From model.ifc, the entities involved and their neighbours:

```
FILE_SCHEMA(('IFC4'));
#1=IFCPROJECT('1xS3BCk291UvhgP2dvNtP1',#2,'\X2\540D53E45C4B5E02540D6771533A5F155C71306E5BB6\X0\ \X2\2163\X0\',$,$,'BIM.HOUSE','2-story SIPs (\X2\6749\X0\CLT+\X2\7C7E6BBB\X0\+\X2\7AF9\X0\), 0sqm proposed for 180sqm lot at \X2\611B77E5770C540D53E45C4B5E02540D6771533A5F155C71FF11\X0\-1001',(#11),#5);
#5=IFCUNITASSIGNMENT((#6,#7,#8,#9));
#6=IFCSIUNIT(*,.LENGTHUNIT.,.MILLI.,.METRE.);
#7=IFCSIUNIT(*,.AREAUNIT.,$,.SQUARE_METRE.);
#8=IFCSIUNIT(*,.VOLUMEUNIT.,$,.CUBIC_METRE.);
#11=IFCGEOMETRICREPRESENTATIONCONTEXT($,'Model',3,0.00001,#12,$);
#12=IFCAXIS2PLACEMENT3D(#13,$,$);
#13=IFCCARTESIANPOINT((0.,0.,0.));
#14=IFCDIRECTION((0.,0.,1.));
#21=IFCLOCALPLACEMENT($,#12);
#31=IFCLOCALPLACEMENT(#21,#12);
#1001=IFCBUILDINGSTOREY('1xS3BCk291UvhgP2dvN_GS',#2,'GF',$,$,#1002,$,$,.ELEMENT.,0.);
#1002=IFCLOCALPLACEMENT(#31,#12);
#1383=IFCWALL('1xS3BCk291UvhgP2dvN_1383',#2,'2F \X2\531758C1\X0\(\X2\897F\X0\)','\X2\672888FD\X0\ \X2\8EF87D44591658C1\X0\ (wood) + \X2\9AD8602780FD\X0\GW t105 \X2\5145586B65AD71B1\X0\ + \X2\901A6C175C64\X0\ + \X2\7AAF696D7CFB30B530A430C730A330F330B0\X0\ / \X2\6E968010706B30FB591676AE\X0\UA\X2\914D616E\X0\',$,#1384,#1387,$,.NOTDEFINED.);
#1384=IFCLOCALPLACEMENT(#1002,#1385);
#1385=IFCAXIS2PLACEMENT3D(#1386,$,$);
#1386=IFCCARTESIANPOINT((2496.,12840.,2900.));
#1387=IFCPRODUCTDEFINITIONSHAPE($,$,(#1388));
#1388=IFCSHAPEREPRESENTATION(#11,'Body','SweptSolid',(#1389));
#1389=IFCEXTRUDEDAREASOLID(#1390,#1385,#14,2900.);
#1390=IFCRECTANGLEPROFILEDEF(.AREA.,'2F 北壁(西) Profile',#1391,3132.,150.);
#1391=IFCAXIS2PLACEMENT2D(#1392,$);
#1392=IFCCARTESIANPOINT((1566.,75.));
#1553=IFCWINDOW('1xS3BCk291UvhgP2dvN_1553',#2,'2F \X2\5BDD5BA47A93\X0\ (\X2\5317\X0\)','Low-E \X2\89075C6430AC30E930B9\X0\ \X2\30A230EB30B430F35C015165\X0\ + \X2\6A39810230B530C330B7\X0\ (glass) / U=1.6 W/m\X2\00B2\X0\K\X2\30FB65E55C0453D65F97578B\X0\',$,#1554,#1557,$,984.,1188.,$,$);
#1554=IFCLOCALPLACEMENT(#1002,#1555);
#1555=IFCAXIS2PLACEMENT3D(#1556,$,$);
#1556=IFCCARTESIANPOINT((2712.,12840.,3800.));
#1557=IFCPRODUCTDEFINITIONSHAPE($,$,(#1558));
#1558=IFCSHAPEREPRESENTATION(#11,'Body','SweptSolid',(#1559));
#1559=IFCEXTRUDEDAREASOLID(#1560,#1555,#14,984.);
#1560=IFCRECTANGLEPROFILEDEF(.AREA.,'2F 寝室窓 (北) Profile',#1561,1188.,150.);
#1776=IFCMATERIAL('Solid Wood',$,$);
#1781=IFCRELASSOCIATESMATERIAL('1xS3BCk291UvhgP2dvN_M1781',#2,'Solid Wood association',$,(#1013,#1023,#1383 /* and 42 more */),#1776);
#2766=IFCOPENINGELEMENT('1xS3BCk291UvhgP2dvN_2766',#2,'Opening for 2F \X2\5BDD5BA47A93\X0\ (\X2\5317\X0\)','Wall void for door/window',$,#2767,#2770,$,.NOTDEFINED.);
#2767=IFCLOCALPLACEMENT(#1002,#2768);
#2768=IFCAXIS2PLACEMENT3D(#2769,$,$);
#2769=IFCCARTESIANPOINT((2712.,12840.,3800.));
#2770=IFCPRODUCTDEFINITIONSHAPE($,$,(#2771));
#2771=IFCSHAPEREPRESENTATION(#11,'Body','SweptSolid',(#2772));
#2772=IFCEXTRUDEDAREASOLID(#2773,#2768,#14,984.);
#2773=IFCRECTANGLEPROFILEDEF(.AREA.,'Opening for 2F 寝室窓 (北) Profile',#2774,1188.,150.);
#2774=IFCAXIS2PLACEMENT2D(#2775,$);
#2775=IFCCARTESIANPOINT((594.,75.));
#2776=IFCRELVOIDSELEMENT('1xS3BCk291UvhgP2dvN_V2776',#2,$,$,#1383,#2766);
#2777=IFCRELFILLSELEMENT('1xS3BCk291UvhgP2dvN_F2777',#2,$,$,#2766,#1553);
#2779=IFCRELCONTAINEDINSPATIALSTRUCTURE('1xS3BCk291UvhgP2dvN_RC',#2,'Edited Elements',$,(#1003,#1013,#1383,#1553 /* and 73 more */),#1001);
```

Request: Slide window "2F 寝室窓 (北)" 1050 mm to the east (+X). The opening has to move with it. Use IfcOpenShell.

```python
import ifcopenshell
import ifcopenshell.api.geometry
import ifcopenshell.util.placement

model = ifcopenshell.open("model.ifc")

window = model.by_guid("1xS3BCk291UvhgP2dvN_1553")
opening = window.FillsVoids[0].RelatingOpeningElement
wall = opening.VoidsElements[0].RelatingBuildingElement

wall_matrix = ifcopenshell.util.placement.get_local_placement(wall.ObjectPlacement)
shift = wall_matrix[:3, 0] * 1050.0
before = ifcopenshell.util.placement.get_local_placement(window.ObjectPlacement)[:3, 3].copy()

# The window is not placed relative to its opening, so move both.
for product in (opening, window):
    matrix = ifcopenshell.util.placement.get_local_placement(product.ObjectPlacement)
    matrix[:3, 3] += shift
    ifcopenshell.api.geometry.edit_object_placement(model, product=product, matrix=matrix, is_si=False)

after = ifcopenshell.util.placement.get_local_placement(window.ObjectPlacement)[:3, 3]
print("window moved by", (after - before).round(3) + 0.0)

model.write("model_rev.ifc")
```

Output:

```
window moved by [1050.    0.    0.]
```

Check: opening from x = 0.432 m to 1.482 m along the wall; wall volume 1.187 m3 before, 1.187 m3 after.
